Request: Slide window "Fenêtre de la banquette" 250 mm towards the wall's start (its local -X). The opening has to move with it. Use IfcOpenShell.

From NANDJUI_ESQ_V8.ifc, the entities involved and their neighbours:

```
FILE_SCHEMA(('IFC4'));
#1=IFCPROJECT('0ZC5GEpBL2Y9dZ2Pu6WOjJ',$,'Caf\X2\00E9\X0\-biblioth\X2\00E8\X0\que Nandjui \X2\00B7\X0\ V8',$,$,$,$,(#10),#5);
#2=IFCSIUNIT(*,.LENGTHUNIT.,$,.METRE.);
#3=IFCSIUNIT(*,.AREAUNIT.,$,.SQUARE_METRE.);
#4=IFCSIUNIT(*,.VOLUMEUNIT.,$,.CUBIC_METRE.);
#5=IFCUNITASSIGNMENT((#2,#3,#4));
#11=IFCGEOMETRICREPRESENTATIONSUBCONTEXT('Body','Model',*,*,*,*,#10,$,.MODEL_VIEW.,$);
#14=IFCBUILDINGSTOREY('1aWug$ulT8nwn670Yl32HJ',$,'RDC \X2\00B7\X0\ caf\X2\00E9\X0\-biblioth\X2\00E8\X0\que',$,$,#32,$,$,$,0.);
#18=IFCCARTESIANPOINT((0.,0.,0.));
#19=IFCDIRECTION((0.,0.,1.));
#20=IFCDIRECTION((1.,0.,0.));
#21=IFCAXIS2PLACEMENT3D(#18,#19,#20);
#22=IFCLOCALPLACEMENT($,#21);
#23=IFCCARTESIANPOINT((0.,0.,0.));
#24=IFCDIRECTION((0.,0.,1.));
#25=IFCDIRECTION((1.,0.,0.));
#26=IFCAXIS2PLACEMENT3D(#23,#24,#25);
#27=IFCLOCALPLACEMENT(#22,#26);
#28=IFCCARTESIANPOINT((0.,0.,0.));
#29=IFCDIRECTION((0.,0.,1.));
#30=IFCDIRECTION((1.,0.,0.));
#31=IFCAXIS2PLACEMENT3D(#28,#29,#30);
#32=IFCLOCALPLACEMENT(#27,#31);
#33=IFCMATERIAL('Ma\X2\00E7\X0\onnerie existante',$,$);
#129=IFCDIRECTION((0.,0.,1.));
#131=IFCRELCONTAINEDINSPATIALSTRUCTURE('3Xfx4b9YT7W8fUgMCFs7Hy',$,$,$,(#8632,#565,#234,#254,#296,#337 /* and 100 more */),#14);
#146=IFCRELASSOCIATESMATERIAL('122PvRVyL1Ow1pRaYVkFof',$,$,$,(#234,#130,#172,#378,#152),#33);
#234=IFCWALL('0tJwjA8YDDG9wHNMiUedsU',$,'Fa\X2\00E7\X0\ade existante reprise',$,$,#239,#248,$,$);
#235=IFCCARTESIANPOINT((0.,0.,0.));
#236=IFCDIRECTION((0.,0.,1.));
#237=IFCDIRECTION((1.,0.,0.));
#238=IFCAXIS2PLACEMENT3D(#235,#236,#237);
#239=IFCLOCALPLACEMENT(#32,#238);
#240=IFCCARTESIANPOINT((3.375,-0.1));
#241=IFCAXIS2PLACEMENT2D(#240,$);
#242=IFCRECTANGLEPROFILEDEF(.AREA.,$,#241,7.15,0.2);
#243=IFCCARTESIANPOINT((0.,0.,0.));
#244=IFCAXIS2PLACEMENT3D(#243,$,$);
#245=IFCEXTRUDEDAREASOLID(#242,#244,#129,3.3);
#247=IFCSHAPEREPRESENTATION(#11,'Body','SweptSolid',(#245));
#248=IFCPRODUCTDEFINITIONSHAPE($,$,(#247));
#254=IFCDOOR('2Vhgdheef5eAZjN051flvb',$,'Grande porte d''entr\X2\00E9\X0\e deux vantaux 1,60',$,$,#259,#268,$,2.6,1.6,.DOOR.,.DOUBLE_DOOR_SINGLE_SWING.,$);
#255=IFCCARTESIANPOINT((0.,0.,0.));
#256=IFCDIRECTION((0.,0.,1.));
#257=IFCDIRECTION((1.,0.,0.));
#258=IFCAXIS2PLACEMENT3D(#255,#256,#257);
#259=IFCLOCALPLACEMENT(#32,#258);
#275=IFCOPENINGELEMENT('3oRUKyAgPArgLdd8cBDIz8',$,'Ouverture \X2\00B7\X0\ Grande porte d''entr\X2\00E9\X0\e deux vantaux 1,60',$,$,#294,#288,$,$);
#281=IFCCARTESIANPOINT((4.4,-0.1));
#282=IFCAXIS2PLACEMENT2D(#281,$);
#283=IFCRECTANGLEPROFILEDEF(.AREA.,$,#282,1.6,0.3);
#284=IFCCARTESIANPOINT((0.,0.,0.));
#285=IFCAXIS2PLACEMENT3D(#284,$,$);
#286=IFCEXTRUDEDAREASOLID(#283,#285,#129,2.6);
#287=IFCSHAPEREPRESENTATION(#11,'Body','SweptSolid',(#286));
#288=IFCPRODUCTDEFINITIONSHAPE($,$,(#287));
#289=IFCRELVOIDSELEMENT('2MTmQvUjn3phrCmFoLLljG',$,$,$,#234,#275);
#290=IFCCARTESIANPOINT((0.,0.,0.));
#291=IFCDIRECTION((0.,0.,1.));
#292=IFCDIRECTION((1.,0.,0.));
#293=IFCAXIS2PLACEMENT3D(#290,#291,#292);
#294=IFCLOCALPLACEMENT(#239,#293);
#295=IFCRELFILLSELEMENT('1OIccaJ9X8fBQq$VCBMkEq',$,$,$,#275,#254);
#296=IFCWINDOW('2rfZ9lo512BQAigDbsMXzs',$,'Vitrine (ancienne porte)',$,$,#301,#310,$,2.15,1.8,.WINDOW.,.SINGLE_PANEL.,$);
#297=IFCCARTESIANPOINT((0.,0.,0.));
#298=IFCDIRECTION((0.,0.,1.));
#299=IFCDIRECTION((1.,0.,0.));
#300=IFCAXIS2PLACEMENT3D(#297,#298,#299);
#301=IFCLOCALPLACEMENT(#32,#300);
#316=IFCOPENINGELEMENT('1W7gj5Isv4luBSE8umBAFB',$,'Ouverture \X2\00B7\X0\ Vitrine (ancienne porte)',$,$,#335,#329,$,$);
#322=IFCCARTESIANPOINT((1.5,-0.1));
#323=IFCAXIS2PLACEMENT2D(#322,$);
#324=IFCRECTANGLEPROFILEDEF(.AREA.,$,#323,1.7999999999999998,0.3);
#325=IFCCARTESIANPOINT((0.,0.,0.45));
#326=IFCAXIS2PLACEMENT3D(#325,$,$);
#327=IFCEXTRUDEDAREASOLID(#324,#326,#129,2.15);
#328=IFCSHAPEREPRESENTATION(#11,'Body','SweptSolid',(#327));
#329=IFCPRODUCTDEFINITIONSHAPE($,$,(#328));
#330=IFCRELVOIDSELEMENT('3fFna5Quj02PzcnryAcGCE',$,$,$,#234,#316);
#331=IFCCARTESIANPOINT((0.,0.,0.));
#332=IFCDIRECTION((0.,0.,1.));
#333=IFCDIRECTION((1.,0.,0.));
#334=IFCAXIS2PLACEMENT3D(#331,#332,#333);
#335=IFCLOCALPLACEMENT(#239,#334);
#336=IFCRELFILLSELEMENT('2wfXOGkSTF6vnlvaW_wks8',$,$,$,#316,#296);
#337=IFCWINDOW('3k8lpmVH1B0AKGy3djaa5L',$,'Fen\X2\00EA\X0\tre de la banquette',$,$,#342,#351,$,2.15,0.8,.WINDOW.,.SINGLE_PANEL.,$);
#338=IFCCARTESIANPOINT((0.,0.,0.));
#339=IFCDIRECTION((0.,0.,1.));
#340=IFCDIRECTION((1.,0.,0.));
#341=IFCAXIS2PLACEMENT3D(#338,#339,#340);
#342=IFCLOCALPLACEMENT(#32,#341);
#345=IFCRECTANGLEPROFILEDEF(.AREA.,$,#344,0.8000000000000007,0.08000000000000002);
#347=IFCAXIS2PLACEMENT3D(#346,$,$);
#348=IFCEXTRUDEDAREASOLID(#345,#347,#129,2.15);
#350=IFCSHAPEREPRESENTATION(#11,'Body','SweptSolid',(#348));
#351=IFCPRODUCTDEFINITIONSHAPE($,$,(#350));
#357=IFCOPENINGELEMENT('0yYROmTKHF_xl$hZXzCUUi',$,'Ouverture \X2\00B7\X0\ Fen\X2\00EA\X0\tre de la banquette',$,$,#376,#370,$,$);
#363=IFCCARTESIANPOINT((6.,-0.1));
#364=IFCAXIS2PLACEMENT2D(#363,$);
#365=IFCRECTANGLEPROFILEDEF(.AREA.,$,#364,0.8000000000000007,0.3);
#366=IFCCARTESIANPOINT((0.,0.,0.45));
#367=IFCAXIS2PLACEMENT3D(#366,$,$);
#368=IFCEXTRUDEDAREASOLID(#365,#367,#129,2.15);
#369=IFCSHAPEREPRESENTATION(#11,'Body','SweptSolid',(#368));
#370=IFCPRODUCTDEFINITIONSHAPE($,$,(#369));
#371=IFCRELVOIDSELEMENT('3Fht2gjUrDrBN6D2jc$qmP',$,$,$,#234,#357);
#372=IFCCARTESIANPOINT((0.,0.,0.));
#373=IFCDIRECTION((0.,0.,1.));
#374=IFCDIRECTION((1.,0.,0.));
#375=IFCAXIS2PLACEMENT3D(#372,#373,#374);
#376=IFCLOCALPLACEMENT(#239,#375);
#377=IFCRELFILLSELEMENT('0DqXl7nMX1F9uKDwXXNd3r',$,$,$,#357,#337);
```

```python
import ifcopenshell
import ifcopenshell.api.geometry
import ifcopenshell.util.placement
import ifcopenshell.util.unit

model = ifcopenshell.open("NANDJUI_ESQ_V8.ifc")
unit_scale = ifcopenshell.util.unit.calculate_unit_scale(model)

window = model.by_guid("3k8lpmVH1B0AKGy3djaa5L")
opening = window.FillsVoids[0].RelatingOpeningElement
wall = opening.VoidsElements[0].RelatingBuildingElement

wall_matrix = ifcopenshell.util.placement.get_local_placement(wall.ObjectPlacement)
shift = wall_matrix[:3, 0] * -0.25 / unit_scale
before = ifcopenshell.util.placement.get_local_placement(window.ObjectPlacement)[:3, 3].copy()

# The window is not placed relative to its opening, so move both.
for product in (opening, window):
    matrix = ifcopenshell.util.placement.get_local_placement(product.ObjectPlacement)
    matrix[:3, 3] += shift
    ifcopenshell.api.geometry.edit_object_placement(model, product=product, matrix=matrix, is_si=False)

after = ifcopenshell.util.placement.get_local_placement(window.ObjectPlacement)[:3, 3]
print("window moved by", (after - before).round(3) + 0.0)

model.write("NANDJUI_ESQ_V8_updated.ifc")
```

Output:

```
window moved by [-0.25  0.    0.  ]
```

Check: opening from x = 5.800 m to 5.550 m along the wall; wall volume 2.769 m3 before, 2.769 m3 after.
